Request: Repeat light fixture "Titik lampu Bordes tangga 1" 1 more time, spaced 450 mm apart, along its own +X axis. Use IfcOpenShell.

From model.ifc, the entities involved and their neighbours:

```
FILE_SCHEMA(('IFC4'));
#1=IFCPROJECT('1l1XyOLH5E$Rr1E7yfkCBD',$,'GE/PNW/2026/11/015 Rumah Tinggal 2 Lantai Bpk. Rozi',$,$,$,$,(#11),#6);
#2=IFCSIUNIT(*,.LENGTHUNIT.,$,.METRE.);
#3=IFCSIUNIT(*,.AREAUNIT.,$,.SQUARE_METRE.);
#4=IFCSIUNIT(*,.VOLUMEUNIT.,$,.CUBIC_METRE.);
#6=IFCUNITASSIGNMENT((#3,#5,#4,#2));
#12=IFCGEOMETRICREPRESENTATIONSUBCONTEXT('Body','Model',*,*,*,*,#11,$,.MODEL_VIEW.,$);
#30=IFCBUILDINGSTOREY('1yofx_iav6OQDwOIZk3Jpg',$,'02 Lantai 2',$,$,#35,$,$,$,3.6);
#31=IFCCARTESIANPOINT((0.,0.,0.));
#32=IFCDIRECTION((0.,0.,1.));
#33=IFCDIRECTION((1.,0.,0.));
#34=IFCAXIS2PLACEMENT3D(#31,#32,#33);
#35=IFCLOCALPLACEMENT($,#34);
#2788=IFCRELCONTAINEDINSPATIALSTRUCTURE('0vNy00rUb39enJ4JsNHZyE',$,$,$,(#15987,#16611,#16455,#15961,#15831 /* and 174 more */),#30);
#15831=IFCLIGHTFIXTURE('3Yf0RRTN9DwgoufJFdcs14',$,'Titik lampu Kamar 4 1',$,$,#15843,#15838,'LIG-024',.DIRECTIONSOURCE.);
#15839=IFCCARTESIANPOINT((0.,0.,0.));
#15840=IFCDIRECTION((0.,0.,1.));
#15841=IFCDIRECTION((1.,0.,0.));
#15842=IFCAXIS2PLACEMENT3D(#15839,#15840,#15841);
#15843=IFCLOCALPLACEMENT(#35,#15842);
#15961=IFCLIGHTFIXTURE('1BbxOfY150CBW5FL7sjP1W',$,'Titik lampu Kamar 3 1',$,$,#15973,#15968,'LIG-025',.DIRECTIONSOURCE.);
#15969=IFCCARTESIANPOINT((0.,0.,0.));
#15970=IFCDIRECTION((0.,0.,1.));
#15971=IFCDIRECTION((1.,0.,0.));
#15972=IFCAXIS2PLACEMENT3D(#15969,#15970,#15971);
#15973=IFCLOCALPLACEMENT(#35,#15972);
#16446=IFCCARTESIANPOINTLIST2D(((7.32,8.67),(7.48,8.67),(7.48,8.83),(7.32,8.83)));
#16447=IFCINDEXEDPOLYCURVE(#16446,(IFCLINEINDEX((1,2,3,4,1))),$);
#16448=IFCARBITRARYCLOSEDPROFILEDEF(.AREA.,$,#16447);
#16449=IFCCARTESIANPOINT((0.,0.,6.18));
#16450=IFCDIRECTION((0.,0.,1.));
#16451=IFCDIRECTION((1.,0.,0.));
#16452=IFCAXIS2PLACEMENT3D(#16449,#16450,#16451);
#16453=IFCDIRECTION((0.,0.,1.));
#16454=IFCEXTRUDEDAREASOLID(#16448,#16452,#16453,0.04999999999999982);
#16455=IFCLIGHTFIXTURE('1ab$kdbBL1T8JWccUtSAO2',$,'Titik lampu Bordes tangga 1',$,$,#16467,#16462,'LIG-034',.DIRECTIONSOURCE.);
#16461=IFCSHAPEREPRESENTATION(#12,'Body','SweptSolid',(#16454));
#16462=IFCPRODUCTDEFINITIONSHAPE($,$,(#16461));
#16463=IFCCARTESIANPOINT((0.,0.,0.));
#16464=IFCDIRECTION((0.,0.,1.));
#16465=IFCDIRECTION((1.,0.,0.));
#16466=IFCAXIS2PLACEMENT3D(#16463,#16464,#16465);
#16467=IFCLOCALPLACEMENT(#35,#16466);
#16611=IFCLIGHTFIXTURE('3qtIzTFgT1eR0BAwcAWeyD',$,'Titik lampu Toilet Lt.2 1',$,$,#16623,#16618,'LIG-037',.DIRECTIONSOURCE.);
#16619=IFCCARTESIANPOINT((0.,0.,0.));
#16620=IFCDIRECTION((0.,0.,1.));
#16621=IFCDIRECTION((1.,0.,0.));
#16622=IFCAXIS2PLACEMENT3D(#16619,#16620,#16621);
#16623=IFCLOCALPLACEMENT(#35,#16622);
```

```python
import ifcopenshell
import ifcopenshell.api.geometry
import ifcopenshell.api.root
import ifcopenshell.util.element
import ifcopenshell.util.placement
import ifcopenshell.util.unit

model = ifcopenshell.open("model.ifc")
unit_scale = ifcopenshell.util.unit.calculate_unit_scale(model)

source = model.by_guid("1ab$kdbBL1T8JWccUtSAO2")
base = ifcopenshell.util.placement.get_local_placement(source.ObjectPlacement)
step = base[:3, 0] * 0.45 / unit_scale

for i in range(1, 2):
    copy = ifcopenshell.api.root.copy_class(model, product=source)
    copy.Representation = ifcopenshell.util.element.copy_deep(
        model, source.Representation, exclude=["IfcGeometricRepresentationContext", "IfcRepresentationMap"]
    )
    copy.Tag = None
    matrix = base.copy()
    matrix[:3, 3] += i * step
    print("added at", matrix[:3, 3].round(3) + 0.0)
    ifcopenshell.api.geometry.edit_object_placement(model, product=copy, matrix=matrix, is_si=False)

model.write("model_edited.ifc")
```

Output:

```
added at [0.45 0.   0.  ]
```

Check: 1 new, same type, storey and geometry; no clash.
